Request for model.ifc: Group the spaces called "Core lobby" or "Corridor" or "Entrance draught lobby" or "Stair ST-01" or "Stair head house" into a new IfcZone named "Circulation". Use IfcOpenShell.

First a look at what the model holds.

```python
import ifcopenshell

model = ifcopenshell.open("model.ifc")
print(model.schema)
seen = {}
for space in model.by_type("IfcSpace"):
    seen[space.LongName] = seen.get(space.LongName, 0) + 1
for name, count in sorted(seen.items(), key=str):
    print(count, "x", name)
print("zones:", [z.Name for z in model.by_type("IfcZone")][:20])
```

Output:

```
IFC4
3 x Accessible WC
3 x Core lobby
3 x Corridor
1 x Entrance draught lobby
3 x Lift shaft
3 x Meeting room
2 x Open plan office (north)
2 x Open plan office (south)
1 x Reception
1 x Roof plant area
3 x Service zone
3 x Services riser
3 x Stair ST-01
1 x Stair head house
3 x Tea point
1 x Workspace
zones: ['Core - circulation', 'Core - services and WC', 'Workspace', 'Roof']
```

```python
import ifcopenshell
import ifcopenshell.api.group
import ifcopenshell.api.root

model = ifcopenshell.open("model.ifc")

names = {"Core lobby", "Corridor", "Entrance draught lobby", "Stair ST-01", "Stair head house"}
spaces = [s for s in model.by_type("IfcSpace") if s.LongName in names]

zone = ifcopenshell.api.root.create_entity(model, ifc_class="IfcZone", name="Circulation")
ifcopenshell.api.group.assign_group(model, products=spaces, group=zone)
print(len(spaces), "spaces in", zone.Name)

model.write("model_edited.ifc")
```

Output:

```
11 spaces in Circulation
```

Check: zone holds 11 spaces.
